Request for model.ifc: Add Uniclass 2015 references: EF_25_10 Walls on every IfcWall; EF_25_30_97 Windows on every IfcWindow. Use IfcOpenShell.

First a look at what the model holds.

```python
import ifcopenshell

model = ifcopenshell.open("model.ifc")
print(model.schema)
print("classifications:", [c.Name for c in model.by_type("IfcClassification")])
for ifc_class in ("IfcDoor", "IfcRoof", "IfcStair", "IfcWall", "IfcWindow"):
    print(ifc_class, len(model.by_type(ifc_class)))
```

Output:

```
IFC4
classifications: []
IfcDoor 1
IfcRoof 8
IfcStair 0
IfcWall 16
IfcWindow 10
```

```python
import ifcopenshell
import ifcopenshell.api.classification

model = ifcopenshell.open("model.ifc")

system = ifcopenshell.api.classification.add_classification(model, classification="Uniclass 2015")

codes = {
    "IfcWall": ("EF_25_10", "Walls"),
    "IfcWindow": ("EF_25_30_97", "Windows"),
}
for ifc_class, (code, name) in codes.items():
    products = model.by_type(ifc_class)
    ifcopenshell.api.classification.add_reference(
        model, products=products, classification=system, identification=code, name=name
    )
    print(code, len(products))

model.write("model_edited.ifc")
```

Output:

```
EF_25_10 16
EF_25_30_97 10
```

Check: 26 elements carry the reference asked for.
